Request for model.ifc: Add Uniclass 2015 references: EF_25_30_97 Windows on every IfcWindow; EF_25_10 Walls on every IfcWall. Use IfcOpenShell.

First a look at what the model holds.

```python
import ifcopenshell

model = ifcopenshell.open("model.ifc")
print(model.schema)
print("classifications:", [c.Name for c in model.by_type("IfcClassification")])
for ifc_class in ("IfcDoor", "IfcRoof", "IfcStair", "IfcWall", "IfcWindow"):
    print(ifc_class, len(model.by_type(ifc_class)))
```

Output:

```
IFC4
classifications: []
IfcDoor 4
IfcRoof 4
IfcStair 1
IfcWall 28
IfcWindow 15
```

```python
import ifcopenshell
import ifcopenshell.api.classification

model = ifcopenshell.open("model.ifc")

system = ifcopenshell.api.classification.add_classification(model, classification="Uniclass 2015")

codes = {
    "IfcWindow": ("EF_25_30_97", "Windows"),
    "IfcWall": ("EF_25_10", "Walls"),
}
for ifc_class, (code, name) in codes.items():
    products = model.by_type(ifc_class)
    ifcopenshell.api.classification.add_reference(
        model, products=products, classification=system, identification=code, name=name
    )
    print(code, len(products))

model.write("model_updated.ifc")
```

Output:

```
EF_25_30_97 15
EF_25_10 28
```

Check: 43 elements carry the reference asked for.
